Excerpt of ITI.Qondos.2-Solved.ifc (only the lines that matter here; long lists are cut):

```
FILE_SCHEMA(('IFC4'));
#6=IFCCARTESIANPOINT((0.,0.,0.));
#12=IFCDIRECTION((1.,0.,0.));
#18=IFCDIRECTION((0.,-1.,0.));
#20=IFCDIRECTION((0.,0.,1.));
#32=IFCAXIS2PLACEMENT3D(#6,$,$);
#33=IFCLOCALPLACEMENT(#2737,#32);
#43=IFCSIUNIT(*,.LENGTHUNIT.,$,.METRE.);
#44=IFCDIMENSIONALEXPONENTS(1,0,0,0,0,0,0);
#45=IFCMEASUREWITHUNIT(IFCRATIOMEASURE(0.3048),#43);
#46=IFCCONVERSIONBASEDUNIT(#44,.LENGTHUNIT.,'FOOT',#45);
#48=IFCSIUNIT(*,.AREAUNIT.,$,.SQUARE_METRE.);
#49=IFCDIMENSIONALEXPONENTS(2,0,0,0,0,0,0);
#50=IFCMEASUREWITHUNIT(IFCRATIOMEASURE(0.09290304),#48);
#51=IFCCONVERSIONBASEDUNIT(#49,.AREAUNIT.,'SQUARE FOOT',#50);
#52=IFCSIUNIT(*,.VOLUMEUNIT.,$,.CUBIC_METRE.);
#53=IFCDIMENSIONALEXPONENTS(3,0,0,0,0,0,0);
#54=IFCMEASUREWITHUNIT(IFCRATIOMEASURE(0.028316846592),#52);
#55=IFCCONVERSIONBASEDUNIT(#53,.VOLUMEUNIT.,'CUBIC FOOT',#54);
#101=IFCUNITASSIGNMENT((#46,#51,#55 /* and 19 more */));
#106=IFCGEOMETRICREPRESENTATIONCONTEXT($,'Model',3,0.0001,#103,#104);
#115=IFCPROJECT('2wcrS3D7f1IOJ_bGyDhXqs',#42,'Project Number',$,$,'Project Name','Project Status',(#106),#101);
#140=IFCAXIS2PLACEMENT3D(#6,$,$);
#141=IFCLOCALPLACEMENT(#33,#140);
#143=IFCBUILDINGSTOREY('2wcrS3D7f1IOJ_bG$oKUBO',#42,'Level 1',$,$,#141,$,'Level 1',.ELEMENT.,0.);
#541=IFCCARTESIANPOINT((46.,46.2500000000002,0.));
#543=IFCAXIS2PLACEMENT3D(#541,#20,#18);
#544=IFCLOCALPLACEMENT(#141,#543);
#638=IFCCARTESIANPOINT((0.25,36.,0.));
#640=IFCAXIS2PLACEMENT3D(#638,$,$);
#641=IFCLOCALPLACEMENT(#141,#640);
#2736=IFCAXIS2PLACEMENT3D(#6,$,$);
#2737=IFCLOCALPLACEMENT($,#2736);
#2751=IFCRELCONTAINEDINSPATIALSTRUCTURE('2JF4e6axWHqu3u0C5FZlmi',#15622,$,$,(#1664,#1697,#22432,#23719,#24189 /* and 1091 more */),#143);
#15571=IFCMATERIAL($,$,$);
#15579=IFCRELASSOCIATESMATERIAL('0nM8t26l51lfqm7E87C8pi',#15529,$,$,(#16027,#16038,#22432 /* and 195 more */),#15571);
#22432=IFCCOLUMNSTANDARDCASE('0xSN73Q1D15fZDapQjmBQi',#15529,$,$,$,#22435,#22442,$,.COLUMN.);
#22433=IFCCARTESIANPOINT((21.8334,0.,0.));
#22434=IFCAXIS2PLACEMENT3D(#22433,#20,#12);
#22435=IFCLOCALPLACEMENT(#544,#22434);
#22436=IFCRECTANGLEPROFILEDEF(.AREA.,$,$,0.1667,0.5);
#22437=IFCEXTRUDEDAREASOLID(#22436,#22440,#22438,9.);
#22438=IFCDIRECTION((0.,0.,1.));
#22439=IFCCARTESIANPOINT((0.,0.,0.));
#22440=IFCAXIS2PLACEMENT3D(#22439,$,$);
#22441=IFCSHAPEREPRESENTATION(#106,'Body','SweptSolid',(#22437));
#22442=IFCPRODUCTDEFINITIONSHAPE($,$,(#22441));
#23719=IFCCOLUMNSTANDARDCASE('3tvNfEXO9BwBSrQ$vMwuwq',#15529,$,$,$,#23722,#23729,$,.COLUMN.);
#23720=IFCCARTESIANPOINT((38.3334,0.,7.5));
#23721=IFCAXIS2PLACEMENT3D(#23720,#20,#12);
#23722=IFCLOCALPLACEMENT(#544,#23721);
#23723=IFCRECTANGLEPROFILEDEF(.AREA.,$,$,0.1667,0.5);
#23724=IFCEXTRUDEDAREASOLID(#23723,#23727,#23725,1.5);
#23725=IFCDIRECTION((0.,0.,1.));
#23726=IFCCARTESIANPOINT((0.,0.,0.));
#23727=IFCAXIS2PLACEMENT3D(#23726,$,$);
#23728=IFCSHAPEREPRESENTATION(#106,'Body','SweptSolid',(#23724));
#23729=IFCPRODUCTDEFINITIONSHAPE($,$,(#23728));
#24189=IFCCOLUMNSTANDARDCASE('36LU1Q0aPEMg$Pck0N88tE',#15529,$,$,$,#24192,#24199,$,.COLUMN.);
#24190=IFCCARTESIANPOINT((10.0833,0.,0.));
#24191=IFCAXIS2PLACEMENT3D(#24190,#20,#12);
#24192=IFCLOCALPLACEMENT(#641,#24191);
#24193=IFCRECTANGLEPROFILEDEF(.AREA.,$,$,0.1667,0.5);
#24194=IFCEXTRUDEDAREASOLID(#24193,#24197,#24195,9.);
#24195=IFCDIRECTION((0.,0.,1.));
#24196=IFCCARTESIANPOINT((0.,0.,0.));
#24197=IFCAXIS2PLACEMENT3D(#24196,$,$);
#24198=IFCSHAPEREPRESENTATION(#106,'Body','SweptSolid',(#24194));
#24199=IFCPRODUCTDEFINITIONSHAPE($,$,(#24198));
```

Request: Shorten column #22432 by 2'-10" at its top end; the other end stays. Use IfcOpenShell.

```python
import ifcopenshell
import ifcopenshell.util.unit

model = ifcopenshell.open("ITI.Qondos.2-Solved.ifc")
unit_scale = ifcopenshell.util.unit.calculate_unit_scale(model)

member = model.by_guid("0xSN73Q1D15fZDapQjmBQi")
change = -34 * 0.0254 / unit_scale

# The extrusion runs towards the end named, so only its depth changes.
body = next(r for r in member.Representation.Representations if r.RepresentationIdentifier == "Body")
solid = body.Items[0]
old_length = solid.Depth
solid.Depth += change

print(f"length {old_length:g} -> {solid.Depth:g}")

model.write("ITI.Qondos.2-Solved_rev.ifc")
```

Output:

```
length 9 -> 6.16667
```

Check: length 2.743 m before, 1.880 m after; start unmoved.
